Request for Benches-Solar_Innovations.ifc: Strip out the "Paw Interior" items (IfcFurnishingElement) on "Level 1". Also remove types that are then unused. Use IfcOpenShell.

First a look at what the model holds.

```python
import ifcopenshell
import ifcopenshell.util.element

model = ifcopenshell.open("Benches-Solar_Innovations.ifc")
print(model.schema)
storey = next(s for s in model.by_type("IfcBuildingStorey") if s.Name == "Level 1")
furniture = [e for e in ifcopenshell.util.element.get_decomposition(storey) if e.is_a("IfcFurnishingElement")]
seen = {}
for e in furniture:
    element_type = ifcopenshell.util.element.get_type(e)
    name = element_type.Name if element_type not in (None, e) else None
    seen[name] = seen.get(name, 0) + 1
for name, count in sorted(seen.items(), key=str):
    print(count, "x", name)
```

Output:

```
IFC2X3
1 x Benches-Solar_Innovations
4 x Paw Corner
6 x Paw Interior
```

```python
import ifcopenshell
import ifcopenshell.api.root
import ifcopenshell.util.element

model = ifcopenshell.open("Benches-Solar_Innovations.ifc")

storey = next(s for s in model.by_type("IfcBuildingStorey") if s.Name == "Level 1")
furniture = [e for e in ifcopenshell.util.element.get_decomposition(storey) if e.is_a("IfcFurnishingElement")]
targets = [e for e in furniture if (t := ifcopenshell.util.element.get_type(e)) not in (None, e) and t.Name == "Paw Interior"]
types = {ifcopenshell.util.element.get_type(e) for e in targets} - {None, *targets}

for e in targets:
    ifcopenshell.api.root.remove_product(model, product=e)
print(len(targets), "removed")

unused = [t for t in types if not ifcopenshell.util.element.get_types(t)]
for t in unused:
    ifcopenshell.api.root.remove_product(model, product=t)
print(len(unused), "unused types removed")

model.write("Benches-Solar_Innovations_rev.ifc")
```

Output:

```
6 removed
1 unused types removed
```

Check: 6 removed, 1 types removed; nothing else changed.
